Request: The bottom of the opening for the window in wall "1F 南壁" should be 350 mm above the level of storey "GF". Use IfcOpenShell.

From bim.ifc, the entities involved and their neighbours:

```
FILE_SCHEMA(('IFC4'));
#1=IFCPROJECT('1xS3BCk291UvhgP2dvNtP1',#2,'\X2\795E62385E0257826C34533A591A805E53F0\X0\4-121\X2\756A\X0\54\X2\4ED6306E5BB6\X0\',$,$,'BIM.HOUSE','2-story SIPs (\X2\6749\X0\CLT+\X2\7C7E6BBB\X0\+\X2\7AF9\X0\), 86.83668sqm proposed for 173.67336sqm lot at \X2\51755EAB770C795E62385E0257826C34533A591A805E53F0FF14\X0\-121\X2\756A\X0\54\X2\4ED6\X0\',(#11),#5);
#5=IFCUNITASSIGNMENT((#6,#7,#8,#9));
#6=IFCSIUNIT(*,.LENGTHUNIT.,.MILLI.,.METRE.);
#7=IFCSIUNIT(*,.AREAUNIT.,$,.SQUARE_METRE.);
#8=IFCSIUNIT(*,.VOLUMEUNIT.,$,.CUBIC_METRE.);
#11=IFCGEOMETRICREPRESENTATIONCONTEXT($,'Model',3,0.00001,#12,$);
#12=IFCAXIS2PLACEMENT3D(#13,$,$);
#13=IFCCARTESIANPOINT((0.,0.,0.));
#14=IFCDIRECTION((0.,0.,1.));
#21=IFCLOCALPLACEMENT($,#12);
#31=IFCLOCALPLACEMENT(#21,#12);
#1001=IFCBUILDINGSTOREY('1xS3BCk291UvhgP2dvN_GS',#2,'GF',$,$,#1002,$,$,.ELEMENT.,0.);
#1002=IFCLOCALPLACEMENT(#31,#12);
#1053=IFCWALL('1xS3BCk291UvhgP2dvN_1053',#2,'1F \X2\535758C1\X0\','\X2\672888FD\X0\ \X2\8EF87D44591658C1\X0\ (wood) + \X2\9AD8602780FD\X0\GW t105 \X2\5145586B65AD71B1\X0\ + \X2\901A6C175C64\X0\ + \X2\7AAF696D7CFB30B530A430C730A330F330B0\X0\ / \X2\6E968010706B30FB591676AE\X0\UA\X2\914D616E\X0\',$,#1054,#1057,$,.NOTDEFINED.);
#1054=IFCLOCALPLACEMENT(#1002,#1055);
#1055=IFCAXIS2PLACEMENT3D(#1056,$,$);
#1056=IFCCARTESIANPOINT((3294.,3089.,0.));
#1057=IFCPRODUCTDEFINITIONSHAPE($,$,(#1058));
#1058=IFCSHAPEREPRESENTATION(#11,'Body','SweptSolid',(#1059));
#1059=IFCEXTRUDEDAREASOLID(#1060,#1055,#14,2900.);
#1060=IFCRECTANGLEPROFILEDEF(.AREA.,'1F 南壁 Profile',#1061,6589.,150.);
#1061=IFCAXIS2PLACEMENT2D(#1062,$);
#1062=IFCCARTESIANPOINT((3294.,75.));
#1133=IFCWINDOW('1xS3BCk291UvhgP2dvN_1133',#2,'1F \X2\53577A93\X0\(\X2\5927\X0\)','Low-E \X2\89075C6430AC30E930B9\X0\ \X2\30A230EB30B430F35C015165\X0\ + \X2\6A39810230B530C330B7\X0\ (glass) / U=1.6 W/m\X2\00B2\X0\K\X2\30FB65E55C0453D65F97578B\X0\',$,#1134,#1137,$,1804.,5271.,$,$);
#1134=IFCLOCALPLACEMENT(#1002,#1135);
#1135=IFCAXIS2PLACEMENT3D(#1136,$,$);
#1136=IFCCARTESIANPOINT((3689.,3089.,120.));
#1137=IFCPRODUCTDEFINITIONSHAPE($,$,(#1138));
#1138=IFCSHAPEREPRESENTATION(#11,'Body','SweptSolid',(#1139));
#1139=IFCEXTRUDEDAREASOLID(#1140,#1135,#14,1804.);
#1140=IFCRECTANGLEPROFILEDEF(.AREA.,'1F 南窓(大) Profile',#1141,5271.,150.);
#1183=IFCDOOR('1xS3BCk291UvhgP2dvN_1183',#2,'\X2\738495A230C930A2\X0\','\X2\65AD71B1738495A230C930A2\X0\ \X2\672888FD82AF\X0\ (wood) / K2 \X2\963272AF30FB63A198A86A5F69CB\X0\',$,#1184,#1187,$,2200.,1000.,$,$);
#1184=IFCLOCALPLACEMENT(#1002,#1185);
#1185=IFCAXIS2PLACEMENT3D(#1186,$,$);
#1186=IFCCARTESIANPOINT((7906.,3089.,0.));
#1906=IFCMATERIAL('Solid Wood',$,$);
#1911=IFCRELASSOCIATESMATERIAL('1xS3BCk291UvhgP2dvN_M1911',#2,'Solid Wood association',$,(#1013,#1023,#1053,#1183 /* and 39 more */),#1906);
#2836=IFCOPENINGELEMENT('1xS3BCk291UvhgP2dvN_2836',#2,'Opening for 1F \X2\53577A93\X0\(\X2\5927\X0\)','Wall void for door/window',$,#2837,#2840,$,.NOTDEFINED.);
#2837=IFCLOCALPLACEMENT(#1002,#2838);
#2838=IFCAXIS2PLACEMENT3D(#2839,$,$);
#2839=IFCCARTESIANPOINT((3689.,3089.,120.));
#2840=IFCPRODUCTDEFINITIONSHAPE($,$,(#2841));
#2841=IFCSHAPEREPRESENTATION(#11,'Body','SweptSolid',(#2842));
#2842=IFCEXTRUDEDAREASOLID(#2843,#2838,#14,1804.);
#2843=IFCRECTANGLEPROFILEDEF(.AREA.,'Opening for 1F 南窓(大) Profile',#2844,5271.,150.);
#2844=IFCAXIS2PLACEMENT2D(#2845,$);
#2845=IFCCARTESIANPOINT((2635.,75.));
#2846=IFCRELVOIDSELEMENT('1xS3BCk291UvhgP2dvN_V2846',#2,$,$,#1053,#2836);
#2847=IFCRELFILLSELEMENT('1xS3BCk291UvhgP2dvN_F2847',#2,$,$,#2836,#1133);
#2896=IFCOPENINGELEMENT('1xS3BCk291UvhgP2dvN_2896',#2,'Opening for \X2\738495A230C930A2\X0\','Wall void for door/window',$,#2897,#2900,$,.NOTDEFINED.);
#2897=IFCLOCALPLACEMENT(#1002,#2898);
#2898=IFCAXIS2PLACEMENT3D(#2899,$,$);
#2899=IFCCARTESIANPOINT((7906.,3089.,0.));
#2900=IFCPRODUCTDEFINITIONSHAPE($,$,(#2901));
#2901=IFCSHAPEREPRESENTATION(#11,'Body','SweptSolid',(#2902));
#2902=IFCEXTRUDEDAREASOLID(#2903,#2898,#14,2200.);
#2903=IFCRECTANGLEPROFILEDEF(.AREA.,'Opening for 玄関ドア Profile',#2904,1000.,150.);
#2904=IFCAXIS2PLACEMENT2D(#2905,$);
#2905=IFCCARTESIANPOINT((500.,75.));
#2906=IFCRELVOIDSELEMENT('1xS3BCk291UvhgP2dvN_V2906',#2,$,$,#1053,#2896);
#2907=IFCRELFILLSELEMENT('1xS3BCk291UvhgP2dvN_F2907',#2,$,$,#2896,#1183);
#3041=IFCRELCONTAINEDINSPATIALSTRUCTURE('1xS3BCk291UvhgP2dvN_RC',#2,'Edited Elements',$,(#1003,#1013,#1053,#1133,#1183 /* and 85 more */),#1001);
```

```python
import numpy as np
import ifcopenshell
import ifcopenshell.api.geometry
import ifcopenshell.geom
import ifcopenshell.util.element
import ifcopenshell.util.placement
import ifcopenshell.util.shape
import ifcopenshell.util.unit

model = ifcopenshell.open("bim.ifc")
unit_scale = ifcopenshell.util.unit.calculate_unit_scale(model)

window = model.by_guid("1xS3BCk291UvhgP2dvN_1133")
opening = window.FillsVoids[0].RelatingOpeningElement
storey = ifcopenshell.util.element.get_container(window, ifc_class="IfcBuildingStorey")
level = ifcopenshell.util.placement.get_local_placement(storey.ObjectPlacement)[2, 3]

# The opening's origin need not be at the sill, so measure its lowest point.
shape = ifcopenshell.geom.create_shape(ifcopenshell.geom.settings(), opening)
bottom = ifcopenshell.util.shape.get_shape_bottom_elevation(shape, shape.geometry) / unit_scale
dz = level + 350.0 - bottom

shift = np.array([0.0, 0.0, dz])
# The window is not placed relative to its opening, so move both.
for product in (opening, window):
    matrix = ifcopenshell.util.placement.get_local_placement(product.ObjectPlacement)
    matrix[:3, 3] += shift
    ifcopenshell.api.geometry.edit_object_placement(model, product=product, matrix=matrix, is_si=False)

print(f"moved by {dz * unit_scale:+.3f} m")

model.write("bim_rev.ifc")
```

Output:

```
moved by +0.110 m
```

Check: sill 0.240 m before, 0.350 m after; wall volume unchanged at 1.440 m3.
